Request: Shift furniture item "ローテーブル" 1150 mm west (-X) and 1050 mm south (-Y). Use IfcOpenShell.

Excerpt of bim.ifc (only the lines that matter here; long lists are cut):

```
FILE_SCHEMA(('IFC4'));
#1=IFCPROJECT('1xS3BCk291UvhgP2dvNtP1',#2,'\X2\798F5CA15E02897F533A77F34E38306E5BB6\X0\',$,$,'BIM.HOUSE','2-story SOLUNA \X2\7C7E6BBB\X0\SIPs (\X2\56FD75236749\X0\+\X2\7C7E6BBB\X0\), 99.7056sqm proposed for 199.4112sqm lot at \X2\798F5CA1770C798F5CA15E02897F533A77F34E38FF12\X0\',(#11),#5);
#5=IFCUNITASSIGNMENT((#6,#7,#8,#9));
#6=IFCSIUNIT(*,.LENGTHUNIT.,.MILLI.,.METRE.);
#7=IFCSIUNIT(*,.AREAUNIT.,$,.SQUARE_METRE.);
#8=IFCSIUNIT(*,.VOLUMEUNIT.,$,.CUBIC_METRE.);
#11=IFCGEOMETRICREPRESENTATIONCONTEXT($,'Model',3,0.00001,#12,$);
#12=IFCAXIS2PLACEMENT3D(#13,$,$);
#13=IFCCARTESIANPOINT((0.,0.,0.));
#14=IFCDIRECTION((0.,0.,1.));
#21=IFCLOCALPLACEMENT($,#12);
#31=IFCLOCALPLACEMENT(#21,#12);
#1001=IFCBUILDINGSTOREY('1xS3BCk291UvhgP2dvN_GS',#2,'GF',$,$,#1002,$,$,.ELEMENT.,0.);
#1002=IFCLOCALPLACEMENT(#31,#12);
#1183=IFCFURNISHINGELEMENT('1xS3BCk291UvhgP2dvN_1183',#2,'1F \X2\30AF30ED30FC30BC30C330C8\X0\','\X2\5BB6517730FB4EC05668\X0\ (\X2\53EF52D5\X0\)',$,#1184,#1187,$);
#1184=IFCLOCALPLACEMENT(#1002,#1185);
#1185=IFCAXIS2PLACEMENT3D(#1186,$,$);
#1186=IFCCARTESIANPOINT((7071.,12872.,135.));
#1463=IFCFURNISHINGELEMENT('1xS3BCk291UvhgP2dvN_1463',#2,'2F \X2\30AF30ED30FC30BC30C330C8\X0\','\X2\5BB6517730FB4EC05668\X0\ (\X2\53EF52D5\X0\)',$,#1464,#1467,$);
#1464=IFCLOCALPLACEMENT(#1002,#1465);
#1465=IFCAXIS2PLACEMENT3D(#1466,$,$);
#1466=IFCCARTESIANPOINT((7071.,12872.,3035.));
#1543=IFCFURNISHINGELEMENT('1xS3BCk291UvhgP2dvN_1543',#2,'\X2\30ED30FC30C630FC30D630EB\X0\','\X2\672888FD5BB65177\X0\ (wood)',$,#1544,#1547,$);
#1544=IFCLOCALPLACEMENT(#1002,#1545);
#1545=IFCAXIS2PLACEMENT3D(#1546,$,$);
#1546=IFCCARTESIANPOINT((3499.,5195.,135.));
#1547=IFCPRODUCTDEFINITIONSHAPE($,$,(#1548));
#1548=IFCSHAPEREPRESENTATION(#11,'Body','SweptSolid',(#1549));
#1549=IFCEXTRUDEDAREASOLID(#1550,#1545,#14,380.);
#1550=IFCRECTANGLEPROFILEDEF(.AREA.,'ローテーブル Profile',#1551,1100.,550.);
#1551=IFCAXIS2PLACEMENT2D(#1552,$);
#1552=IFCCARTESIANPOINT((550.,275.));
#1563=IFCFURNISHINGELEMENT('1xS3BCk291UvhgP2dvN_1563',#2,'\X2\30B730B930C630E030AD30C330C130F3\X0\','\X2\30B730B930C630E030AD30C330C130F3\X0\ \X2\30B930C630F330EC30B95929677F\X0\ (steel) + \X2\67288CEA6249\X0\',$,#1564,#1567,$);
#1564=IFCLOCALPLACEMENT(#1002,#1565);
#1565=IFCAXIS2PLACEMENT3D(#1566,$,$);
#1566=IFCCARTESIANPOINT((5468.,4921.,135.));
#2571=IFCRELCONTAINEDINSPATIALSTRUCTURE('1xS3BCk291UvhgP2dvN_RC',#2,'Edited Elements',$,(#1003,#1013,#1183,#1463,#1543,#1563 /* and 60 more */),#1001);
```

```python
import ifcopenshell
import ifcopenshell.api.geometry
import ifcopenshell.util.placement

model = ifcopenshell.open("bim.ifc")

item = model.by_guid("1xS3BCk291UvhgP2dvN_1543")
matrix = ifcopenshell.util.placement.get_local_placement(item.ObjectPlacement)
matrix[0, 3] -= 1150.0
matrix[1, 3] -= 1050.0
ifcopenshell.api.geometry.edit_object_placement(model, product=item, matrix=matrix, is_si=False)

print(ifcopenshell.util.placement.get_local_placement(item.ObjectPlacement).round(3) + 0.0)

model.write("bim_rev.ifc")
```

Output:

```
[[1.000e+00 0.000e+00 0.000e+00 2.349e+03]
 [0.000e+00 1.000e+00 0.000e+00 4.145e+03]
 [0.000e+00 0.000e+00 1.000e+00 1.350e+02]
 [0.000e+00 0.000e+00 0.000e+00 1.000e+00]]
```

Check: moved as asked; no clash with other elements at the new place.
